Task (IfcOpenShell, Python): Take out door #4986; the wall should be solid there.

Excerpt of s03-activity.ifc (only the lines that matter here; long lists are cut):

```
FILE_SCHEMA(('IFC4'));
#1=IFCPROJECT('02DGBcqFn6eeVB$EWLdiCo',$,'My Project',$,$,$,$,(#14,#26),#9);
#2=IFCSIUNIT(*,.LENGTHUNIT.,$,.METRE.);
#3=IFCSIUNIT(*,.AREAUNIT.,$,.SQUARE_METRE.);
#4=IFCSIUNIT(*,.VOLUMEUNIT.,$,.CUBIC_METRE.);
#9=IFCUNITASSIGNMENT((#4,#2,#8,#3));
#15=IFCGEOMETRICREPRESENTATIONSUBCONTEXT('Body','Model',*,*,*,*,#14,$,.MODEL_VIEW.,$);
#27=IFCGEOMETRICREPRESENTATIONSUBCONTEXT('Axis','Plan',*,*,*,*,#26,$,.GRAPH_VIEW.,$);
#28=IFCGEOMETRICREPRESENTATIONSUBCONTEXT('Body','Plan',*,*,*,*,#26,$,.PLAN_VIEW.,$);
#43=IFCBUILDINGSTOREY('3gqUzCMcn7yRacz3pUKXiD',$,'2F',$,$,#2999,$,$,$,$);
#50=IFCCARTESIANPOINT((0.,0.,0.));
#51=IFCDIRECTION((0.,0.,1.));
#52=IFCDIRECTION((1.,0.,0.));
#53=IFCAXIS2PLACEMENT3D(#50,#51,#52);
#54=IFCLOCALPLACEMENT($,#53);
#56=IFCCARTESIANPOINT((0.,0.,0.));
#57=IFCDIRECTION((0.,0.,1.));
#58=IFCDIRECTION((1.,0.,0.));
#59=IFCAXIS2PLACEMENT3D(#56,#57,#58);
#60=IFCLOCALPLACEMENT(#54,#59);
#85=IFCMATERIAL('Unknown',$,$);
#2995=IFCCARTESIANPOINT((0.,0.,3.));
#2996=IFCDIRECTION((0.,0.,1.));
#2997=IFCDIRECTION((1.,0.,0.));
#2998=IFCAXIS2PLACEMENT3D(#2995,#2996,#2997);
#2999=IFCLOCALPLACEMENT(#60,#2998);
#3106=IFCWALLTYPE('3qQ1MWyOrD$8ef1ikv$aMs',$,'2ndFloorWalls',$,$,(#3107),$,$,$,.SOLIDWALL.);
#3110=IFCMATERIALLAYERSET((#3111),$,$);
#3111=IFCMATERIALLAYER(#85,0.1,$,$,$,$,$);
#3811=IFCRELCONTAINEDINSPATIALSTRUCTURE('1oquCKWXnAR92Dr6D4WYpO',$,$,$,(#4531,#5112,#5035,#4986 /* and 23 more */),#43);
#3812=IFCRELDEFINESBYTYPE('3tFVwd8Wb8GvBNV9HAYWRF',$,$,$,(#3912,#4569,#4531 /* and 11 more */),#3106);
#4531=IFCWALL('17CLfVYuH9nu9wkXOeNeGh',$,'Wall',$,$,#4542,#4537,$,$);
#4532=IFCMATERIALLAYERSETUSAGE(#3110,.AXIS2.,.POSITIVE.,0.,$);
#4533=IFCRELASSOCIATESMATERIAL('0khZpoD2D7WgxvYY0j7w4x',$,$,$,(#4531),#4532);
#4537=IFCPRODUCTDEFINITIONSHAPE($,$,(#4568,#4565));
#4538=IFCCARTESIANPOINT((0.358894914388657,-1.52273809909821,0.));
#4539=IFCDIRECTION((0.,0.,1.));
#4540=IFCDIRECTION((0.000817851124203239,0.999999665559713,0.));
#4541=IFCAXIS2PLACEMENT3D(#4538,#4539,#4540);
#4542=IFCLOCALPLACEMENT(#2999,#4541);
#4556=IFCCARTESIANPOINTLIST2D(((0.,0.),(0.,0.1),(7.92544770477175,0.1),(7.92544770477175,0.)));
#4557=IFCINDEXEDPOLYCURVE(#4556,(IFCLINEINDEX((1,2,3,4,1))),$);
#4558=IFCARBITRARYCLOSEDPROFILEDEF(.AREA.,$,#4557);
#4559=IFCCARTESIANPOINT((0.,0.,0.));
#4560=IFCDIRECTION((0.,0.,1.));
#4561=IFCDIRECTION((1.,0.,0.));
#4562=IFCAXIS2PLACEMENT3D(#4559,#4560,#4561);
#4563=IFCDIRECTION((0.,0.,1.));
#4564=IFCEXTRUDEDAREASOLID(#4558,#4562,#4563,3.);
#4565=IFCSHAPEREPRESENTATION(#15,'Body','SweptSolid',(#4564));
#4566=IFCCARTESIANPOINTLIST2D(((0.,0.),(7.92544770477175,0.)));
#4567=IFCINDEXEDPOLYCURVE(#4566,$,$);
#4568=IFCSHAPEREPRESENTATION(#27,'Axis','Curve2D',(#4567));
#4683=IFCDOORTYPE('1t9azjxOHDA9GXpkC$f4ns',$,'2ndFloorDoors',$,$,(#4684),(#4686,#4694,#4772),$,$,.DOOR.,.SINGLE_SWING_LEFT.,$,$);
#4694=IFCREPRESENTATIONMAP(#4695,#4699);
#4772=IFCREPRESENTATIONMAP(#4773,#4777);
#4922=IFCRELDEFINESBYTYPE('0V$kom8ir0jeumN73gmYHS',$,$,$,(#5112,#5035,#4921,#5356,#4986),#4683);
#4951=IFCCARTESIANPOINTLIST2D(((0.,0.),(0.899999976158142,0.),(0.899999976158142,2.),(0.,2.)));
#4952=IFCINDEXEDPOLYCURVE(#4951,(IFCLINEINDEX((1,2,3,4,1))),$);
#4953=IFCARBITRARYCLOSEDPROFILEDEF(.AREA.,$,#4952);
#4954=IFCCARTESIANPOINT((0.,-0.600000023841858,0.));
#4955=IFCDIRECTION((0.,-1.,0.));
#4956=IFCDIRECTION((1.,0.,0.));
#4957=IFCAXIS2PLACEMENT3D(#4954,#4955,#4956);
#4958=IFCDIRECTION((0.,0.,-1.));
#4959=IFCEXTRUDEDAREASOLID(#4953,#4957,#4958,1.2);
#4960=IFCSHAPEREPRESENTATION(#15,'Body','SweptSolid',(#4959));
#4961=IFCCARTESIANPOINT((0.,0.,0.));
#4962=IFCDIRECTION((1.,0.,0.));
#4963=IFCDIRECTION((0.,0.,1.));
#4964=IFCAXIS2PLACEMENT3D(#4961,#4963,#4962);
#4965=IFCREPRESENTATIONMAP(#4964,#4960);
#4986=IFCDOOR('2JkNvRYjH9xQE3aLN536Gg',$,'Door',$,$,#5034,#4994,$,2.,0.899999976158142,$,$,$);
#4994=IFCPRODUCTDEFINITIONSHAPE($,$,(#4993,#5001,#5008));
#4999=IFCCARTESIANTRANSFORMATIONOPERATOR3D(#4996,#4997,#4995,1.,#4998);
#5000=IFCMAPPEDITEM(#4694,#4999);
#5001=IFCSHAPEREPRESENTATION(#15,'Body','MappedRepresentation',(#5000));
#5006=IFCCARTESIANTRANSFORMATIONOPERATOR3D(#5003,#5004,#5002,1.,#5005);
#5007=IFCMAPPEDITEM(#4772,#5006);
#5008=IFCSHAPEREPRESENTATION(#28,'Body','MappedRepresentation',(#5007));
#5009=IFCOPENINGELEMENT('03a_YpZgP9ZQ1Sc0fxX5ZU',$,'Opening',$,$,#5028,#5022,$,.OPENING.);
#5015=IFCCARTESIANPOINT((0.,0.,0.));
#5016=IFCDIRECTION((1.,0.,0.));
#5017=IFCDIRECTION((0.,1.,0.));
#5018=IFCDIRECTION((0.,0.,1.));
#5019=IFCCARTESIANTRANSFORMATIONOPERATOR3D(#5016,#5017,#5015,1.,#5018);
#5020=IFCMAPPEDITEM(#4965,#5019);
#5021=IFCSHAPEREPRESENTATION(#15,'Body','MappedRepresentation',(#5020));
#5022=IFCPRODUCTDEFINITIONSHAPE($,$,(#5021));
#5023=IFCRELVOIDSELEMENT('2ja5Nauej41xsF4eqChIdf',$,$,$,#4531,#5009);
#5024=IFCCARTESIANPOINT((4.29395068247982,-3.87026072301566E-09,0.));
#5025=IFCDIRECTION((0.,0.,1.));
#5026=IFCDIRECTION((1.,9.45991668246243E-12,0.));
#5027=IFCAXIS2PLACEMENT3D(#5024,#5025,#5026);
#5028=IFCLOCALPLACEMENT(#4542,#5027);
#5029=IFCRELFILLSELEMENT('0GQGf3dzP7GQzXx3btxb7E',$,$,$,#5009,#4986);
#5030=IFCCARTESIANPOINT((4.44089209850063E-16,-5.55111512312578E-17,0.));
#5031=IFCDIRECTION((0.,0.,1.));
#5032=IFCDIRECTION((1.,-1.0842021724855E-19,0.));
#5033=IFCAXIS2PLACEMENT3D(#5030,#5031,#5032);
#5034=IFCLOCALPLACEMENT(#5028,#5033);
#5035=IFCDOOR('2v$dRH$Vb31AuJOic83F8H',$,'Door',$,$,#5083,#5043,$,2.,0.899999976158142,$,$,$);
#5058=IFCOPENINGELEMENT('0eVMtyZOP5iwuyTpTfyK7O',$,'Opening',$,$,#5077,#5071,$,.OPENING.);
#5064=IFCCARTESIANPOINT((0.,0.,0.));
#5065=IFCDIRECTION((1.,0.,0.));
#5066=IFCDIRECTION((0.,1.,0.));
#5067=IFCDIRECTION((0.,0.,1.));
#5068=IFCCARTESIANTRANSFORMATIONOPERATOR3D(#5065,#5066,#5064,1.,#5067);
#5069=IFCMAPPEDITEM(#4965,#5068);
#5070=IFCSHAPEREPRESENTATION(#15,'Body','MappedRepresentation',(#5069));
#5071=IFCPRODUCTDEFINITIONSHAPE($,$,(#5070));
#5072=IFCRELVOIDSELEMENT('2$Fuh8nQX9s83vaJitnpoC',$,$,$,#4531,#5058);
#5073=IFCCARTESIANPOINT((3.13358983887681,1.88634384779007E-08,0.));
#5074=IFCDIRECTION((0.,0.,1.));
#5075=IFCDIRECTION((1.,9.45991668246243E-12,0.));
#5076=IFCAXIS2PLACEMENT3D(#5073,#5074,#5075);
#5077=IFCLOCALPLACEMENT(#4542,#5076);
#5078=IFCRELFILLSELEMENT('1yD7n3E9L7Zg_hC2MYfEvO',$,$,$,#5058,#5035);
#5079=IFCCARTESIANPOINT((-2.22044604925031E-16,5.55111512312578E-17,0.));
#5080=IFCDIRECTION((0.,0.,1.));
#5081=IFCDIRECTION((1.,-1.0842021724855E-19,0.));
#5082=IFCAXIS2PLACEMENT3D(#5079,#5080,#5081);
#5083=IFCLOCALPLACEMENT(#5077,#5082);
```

```python
import ifcopenshell
import ifcopenshell.api.feature
import ifcopenshell.api.root
import ifcopenshell.geom
import ifcopenshell.util.shape

model = ifcopenshell.open("s03-activity.ifc")
settings = ifcopenshell.geom.settings()


def volume(element):
    """Net volume in cubic metres, openings subtracted."""
    shape = ifcopenshell.geom.create_shape(settings, element)
    return ifcopenshell.util.shape.get_volume(shape.geometry)


door = model.by_guid("2JkNvRYjH9xQE3aLN536Gg")
opening = door.FillsVoids[0].RelatingOpeningElement
wall = opening.VoidsElements[0].RelatingBuildingElement
before = volume(wall)

ifcopenshell.api.root.remove_product(model, product=door)
ifcopenshell.api.feature.remove_feature(model, feature=opening)

after = volume(wall)

print(f"wall volume {before:.3f} -> {after:.3f} m3")

model.write("s03-activity_v2.ifc")
```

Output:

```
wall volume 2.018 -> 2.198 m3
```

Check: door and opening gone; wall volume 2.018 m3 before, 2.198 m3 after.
